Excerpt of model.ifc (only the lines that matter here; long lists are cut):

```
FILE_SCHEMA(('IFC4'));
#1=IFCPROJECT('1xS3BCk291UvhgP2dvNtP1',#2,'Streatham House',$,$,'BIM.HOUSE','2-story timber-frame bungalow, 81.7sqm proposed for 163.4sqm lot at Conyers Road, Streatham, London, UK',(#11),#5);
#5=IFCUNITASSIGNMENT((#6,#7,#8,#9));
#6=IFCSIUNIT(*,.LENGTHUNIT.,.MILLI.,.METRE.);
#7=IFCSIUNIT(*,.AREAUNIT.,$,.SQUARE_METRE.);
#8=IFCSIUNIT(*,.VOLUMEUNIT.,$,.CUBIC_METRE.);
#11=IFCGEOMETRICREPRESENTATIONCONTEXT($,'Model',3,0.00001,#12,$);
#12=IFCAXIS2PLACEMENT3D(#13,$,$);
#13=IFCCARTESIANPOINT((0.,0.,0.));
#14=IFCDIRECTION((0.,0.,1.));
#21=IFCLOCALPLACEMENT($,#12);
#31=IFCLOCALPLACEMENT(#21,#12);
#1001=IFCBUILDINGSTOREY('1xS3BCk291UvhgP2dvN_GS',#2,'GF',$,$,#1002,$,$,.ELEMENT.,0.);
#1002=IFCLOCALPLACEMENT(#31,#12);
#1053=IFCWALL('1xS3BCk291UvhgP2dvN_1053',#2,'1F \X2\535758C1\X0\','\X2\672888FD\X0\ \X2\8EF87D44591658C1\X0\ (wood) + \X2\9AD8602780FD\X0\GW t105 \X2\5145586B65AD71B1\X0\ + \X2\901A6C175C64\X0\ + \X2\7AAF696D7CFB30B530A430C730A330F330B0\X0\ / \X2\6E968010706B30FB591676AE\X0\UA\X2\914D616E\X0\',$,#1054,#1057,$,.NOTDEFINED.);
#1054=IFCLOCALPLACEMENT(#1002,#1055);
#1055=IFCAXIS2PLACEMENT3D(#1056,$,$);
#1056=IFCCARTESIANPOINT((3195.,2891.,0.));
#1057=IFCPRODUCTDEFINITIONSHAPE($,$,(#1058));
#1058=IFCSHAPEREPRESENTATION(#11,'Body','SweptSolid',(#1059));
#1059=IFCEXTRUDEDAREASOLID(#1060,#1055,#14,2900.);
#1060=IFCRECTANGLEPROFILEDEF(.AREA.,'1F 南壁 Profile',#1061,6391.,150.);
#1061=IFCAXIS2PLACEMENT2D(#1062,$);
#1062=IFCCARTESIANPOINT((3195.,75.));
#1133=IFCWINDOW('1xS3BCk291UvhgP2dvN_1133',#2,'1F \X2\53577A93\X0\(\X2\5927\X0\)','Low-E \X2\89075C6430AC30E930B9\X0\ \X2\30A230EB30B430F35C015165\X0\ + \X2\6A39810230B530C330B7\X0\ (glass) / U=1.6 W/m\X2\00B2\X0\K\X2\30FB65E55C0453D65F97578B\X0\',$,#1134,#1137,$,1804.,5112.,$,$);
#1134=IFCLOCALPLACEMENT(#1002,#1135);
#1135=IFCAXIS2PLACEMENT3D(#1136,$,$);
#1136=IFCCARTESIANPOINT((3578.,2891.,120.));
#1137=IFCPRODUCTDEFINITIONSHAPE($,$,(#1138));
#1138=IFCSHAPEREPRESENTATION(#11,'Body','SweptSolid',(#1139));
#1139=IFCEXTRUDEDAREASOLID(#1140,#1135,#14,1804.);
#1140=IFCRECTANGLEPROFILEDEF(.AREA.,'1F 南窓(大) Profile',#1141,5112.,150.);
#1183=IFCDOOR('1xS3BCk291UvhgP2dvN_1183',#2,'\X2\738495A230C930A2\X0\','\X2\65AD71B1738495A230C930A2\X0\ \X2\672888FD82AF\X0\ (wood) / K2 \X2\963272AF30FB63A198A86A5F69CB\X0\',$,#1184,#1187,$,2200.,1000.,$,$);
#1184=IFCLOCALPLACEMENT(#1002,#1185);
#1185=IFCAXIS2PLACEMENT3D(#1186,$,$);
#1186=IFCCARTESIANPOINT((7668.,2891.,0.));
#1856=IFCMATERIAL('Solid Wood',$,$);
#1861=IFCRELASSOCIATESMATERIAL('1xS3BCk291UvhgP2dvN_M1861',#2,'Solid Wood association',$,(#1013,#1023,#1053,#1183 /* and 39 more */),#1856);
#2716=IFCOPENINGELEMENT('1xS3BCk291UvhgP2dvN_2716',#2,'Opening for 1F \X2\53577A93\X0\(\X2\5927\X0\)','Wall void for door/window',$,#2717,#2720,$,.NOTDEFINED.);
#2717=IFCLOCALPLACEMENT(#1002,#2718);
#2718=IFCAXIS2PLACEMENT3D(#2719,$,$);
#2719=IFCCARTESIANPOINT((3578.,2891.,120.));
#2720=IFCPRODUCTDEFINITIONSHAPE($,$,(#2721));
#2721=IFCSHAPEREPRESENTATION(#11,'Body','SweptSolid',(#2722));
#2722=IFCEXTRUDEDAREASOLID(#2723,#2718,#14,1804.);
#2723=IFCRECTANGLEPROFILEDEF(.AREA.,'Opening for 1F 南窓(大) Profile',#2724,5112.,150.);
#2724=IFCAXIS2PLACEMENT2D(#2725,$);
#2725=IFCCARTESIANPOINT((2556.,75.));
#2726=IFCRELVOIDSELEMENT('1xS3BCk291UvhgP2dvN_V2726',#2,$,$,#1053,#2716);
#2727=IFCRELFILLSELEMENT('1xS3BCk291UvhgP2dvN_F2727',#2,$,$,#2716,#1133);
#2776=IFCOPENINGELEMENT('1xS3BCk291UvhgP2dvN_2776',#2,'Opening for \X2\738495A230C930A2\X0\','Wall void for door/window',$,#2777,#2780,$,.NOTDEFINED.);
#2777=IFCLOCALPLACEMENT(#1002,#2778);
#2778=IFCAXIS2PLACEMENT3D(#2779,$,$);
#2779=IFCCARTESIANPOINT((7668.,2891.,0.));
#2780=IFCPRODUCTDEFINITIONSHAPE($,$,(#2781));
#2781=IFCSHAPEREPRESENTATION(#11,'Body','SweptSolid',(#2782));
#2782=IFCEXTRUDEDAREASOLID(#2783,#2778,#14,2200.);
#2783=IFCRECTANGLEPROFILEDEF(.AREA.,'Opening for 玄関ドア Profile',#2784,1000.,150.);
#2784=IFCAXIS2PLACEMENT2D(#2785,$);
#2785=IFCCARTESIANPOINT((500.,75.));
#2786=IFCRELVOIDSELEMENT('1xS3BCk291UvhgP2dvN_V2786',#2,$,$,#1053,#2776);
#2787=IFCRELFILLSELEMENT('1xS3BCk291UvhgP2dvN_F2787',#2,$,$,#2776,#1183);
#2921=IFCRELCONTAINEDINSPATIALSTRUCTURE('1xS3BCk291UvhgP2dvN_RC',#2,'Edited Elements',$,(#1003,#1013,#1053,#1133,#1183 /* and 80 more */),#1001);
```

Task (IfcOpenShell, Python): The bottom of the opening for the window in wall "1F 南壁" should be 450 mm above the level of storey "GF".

```python
import numpy as np
import ifcopenshell
import ifcopenshell.api.geometry
import ifcopenshell.geom
import ifcopenshell.util.element
import ifcopenshell.util.placement
import ifcopenshell.util.shape
import ifcopenshell.util.unit

model = ifcopenshell.open("model.ifc")
unit_scale = ifcopenshell.util.unit.calculate_unit_scale(model)

window = model.by_guid("1xS3BCk291UvhgP2dvN_1133")
opening = window.FillsVoids[0].RelatingOpeningElement
storey = ifcopenshell.util.element.get_container(window, ifc_class="IfcBuildingStorey")
level = ifcopenshell.util.placement.get_local_placement(storey.ObjectPlacement)[2, 3]

# The opening's origin need not be at the sill, so measure its lowest point.
shape = ifcopenshell.geom.create_shape(ifcopenshell.geom.settings(), opening)
bottom = ifcopenshell.util.shape.get_shape_bottom_elevation(shape, shape.geometry) / unit_scale
dz = level + 0.45 / unit_scale - bottom

shift = np.array([0.0, 0.0, dz])
# The window is not placed relative to its opening, so move both.
for product in (opening, window):
    matrix = ifcopenshell.util.placement.get_local_placement(product.ObjectPlacement)
    matrix[:3, 3] += shift
    ifcopenshell.api.geometry.edit_object_placement(model, product=product, matrix=matrix, is_si=False)

print(f"moved by {dz * unit_scale:+.3f} m")

model.write("model_v2.ifc")
```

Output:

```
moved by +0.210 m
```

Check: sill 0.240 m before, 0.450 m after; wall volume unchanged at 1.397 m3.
